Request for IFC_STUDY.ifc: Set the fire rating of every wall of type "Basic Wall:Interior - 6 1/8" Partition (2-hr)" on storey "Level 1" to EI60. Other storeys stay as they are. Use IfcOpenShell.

First a look at what the model holds.

```python
import ifcopenshell
import ifcopenshell.util.element

model = ifcopenshell.open("IFC_STUDY.ifc")
print(model.schema)
storey = next(s for s in model.by_type("IfcBuildingStorey") if s.Name == "Level 1")
walls = [e for e in ifcopenshell.util.element.get_decomposition(storey) if e.is_a("IfcWall")]
seen = {}
for e in walls:
    element_type = ifcopenshell.util.element.get_type(e)
    key = (element_type.Name if element_type != e and element_type else None, ifcopenshell.util.element.get_pset(e, "Pset_WallCommon", "FireRating"))
    seen[key] = seen.get(key, 0) + 1
for (name, value), count in sorted(seen.items(), key=str):
    print(count, "x", name, "|", value)
```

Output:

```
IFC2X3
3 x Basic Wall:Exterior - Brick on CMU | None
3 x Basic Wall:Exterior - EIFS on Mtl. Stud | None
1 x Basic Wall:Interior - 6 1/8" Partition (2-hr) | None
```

```python
import ifcopenshell
import ifcopenshell.api.pset
import ifcopenshell.util.element

model = ifcopenshell.open("IFC_STUDY.ifc")

storey = next(s for s in model.by_type("IfcBuildingStorey") if s.Name == "Level 1")
walls = [e for e in ifcopenshell.util.element.get_decomposition(storey) if e.is_a("IfcWall")]

count = 0
for e in walls:
    element_type = ifcopenshell.util.element.get_type(e)
    if element_type in (None, e) or element_type.Name != 'Basic Wall:Interior - 6 1/8" Partition (2-hr)':
        continue
    # add_pset returns the element's existing set when there is one.
    pset = ifcopenshell.api.pset.add_pset(model, product=e, name="Pset_WallCommon")
    ifcopenshell.api.pset.edit_pset(model, pset=pset, properties={"FireRating": "EI60"})
    count += 1

print(count, "walls updated")

model.write("IFC_STUDY-out.ifc")
```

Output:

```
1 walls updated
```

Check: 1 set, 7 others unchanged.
